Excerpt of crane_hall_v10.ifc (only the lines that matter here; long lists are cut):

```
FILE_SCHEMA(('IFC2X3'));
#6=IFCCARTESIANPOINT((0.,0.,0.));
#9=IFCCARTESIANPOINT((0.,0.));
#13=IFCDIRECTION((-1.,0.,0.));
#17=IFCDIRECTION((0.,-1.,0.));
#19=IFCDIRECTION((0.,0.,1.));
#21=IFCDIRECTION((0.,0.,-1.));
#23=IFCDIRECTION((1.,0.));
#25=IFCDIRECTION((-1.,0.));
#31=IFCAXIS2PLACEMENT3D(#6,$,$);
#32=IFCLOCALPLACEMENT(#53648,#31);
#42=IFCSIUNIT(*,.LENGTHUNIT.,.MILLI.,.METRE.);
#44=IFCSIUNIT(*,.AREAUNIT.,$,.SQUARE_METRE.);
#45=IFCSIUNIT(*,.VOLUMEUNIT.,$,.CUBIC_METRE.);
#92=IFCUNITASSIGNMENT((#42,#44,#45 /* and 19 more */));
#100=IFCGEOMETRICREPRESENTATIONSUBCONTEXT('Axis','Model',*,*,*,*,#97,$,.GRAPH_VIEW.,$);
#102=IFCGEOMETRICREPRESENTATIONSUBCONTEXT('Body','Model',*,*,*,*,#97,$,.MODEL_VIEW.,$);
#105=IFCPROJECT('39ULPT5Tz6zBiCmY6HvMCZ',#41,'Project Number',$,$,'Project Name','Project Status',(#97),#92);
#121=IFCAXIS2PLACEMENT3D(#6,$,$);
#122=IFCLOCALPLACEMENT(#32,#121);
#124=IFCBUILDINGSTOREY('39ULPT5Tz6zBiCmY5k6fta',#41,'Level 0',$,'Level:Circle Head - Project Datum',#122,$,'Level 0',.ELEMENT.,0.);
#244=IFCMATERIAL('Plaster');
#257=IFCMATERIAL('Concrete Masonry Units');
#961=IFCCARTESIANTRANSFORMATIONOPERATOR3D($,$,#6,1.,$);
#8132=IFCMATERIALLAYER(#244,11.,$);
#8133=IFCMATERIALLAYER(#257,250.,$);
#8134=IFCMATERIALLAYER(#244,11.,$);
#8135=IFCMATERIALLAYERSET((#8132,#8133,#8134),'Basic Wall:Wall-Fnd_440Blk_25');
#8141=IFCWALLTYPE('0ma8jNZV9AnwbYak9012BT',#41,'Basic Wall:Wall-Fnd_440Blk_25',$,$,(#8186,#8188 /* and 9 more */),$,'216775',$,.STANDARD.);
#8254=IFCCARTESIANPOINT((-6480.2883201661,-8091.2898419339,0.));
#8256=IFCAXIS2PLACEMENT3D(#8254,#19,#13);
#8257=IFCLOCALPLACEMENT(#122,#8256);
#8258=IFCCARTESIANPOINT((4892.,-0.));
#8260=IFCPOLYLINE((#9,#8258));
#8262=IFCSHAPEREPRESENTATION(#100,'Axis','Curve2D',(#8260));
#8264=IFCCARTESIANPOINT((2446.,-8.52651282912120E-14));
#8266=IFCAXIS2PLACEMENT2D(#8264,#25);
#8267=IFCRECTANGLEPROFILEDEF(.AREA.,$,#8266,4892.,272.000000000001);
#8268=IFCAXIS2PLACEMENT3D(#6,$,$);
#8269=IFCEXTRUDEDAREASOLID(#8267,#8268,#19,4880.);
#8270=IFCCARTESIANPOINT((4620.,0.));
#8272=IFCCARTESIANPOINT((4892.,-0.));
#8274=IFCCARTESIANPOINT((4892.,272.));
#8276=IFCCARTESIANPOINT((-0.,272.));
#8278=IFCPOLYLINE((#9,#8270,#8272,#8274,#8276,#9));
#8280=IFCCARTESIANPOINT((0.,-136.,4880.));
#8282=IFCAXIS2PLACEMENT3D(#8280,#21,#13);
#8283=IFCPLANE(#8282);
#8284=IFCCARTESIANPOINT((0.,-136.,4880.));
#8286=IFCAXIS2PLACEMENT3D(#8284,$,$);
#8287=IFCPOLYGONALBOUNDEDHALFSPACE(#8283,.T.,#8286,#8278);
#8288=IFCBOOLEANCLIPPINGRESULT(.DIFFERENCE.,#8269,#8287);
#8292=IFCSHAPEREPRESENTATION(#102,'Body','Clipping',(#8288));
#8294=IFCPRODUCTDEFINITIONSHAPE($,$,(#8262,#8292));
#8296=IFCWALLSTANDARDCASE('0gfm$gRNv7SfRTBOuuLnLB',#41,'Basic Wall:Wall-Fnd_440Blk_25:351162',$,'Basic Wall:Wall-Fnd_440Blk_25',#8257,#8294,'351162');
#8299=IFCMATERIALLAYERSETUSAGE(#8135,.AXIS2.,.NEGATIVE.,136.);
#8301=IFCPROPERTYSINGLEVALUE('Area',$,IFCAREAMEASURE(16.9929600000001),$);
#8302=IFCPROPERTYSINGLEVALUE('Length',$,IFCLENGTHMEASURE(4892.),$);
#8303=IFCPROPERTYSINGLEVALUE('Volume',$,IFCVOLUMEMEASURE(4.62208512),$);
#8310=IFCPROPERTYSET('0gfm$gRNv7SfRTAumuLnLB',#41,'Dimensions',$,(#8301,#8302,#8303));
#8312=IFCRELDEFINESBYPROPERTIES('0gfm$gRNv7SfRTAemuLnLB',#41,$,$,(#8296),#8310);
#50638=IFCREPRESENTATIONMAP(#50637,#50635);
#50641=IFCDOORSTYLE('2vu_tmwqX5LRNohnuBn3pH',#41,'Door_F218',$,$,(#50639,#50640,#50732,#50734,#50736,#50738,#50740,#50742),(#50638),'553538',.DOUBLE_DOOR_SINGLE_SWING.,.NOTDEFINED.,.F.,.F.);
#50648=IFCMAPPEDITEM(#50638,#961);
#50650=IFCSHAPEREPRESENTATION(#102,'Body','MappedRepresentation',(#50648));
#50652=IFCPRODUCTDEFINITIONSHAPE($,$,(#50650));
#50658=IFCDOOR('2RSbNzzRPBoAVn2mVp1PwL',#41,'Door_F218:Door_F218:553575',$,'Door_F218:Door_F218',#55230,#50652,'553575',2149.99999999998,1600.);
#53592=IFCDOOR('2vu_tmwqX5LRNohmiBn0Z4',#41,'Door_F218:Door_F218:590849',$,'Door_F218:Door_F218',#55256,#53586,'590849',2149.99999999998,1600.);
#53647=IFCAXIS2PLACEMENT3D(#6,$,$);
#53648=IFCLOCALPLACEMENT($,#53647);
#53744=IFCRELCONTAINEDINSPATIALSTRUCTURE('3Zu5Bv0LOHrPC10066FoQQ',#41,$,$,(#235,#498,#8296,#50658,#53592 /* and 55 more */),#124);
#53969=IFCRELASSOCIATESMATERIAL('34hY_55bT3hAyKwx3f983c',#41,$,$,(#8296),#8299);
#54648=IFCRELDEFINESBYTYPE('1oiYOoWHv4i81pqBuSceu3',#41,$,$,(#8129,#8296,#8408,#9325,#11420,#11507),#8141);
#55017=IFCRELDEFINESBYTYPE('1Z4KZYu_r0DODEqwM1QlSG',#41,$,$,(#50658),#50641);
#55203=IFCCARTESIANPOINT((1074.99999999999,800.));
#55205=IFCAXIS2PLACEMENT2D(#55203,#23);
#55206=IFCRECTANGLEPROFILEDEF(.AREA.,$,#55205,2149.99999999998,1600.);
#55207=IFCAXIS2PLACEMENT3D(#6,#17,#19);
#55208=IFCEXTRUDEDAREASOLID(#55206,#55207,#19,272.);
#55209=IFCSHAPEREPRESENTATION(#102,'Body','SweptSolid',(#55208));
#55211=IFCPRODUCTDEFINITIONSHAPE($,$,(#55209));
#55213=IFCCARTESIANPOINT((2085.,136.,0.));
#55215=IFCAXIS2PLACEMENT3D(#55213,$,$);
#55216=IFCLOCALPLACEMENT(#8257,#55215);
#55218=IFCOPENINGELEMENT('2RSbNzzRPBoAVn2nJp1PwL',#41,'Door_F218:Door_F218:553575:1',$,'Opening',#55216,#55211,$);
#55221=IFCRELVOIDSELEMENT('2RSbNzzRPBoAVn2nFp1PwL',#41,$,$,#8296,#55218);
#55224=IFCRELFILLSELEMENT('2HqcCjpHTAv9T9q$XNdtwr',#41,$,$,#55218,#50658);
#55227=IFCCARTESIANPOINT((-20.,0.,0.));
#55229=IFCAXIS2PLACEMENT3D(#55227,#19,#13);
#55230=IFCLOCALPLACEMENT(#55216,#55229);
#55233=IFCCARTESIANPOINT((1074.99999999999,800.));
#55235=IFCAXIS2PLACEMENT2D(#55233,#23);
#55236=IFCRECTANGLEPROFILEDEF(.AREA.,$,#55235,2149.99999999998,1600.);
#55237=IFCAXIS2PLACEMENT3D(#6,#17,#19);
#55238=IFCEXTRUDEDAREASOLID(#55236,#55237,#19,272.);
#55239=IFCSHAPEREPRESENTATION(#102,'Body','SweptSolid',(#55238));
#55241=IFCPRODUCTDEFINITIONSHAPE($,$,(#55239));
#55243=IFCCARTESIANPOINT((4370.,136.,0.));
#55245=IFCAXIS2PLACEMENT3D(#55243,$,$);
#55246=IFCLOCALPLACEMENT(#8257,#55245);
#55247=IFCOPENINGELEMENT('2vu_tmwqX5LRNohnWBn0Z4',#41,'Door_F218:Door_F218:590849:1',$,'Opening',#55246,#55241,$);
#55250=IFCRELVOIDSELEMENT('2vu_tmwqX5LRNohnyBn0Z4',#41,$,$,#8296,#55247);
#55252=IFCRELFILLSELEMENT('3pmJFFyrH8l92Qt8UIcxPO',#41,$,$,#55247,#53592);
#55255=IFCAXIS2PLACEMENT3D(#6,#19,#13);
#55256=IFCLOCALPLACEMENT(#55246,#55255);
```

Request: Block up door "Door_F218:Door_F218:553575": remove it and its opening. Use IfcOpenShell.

```python
import ifcopenshell
import ifcopenshell.api.feature
import ifcopenshell.api.pset
import ifcopenshell.api.root
import ifcopenshell.geom
import ifcopenshell.util.element
import ifcopenshell.util.shape
import ifcopenshell.util.unit

model = ifcopenshell.open("crane_hall_v10.ifc")
area_scale = ifcopenshell.util.unit.calculate_unit_scale(model, "AREAUNIT")
volume_scale = ifcopenshell.util.unit.calculate_unit_scale(model, "VOLUMEUNIT")
settings = ifcopenshell.geom.settings()


def volume(element):
    """Net volume in cubic metres, openings subtracted."""
    shape = ifcopenshell.geom.create_shape(settings, element)
    return ifcopenshell.util.shape.get_volume(shape.geometry)


door = model.by_guid("2RSbNzzRPBoAVn2mVp1PwL")
opening = door.FillsVoids[0].RelatingOpeningElement
wall = opening.VoidsElements[0].RelatingBuildingElement
before = volume(wall)

ifcopenshell.api.root.remove_product(model, product=door)
ifcopenshell.api.feature.remove_feature(model, feature=opening)

after = volume(wall)
thickness = 0.272  # wall thickness in metres

# Update the wall's stored quantities.
pset = model.by_id(ifcopenshell.util.element.get_pset(wall, "Dimensions", should_inherit=False)["id"])
ifcopenshell.api.pset.edit_pset(model, pset=pset, properties={
    "Area": model.create_entity("IfcAreaMeasure", after / thickness / area_scale),
    "Volume": model.create_entity("IfcVolumeMeasure", after / volume_scale),
})

print(f"wall volume {before:.3f} -> {after:.3f} m3")

model.write("crane_hall_v10-out.ifc")
```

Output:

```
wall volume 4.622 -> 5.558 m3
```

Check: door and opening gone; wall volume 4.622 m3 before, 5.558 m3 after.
